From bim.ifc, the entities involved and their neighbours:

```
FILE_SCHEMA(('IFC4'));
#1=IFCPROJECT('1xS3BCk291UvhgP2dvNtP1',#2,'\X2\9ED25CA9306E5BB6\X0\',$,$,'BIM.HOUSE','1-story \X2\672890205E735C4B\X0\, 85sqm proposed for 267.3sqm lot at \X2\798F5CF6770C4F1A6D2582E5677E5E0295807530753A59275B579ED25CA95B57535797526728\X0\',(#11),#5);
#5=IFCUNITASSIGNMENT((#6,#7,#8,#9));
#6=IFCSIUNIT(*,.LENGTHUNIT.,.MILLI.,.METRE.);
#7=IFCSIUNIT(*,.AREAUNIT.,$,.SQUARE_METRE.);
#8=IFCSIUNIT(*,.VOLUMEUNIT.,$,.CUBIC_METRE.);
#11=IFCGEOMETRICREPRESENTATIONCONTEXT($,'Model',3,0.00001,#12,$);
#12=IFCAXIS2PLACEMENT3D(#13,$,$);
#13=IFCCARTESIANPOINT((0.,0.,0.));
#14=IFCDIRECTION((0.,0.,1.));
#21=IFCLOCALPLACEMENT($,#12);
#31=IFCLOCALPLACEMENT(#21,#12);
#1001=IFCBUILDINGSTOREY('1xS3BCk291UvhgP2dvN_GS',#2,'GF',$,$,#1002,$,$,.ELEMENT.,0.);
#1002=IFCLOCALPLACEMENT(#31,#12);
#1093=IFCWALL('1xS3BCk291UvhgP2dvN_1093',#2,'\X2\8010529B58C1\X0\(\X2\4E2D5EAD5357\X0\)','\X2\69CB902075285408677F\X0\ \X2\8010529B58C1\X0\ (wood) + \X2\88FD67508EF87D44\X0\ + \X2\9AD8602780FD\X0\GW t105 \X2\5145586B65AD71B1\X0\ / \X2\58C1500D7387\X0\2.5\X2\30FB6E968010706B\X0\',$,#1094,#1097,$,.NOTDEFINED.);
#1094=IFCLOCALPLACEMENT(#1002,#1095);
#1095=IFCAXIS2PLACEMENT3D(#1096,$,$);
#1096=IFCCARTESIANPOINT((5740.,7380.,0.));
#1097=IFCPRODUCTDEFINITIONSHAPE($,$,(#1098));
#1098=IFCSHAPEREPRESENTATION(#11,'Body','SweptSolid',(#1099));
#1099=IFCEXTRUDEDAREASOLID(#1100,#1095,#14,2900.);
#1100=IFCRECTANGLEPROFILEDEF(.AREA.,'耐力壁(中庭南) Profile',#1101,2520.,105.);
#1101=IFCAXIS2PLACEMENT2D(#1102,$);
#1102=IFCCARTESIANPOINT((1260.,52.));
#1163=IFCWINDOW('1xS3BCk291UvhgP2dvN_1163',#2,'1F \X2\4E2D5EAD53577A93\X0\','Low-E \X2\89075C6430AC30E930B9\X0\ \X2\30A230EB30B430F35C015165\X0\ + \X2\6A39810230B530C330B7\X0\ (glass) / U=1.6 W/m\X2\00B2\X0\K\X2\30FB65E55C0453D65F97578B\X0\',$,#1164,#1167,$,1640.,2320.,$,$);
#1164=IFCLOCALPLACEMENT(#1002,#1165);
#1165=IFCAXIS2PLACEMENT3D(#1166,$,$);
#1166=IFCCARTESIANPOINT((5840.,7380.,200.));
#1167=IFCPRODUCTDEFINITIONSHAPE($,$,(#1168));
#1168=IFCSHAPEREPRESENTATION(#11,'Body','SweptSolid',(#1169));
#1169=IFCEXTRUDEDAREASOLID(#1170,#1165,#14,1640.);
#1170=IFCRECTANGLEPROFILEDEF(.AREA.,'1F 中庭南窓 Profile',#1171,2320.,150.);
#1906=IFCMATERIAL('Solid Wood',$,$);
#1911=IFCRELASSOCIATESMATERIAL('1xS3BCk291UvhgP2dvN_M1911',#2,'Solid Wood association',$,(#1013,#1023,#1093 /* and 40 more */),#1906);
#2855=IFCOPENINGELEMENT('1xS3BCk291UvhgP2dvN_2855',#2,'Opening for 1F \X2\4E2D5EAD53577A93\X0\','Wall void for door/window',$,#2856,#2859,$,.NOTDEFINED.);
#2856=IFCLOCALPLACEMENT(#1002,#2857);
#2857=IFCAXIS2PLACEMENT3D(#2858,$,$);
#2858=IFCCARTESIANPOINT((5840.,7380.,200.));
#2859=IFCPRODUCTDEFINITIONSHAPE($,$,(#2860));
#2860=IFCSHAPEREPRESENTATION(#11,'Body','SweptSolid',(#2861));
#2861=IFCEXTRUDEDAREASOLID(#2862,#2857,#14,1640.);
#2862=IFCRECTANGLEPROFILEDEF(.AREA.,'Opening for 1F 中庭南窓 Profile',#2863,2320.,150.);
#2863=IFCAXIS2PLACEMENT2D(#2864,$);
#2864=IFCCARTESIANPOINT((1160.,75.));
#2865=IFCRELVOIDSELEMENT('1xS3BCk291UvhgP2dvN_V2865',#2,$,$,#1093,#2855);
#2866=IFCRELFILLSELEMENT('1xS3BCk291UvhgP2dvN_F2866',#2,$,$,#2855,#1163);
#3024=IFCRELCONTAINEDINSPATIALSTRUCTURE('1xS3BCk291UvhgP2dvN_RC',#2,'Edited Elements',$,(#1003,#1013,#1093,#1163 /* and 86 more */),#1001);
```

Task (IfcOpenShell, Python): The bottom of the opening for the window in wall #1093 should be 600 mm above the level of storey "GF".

```python
import numpy as np
import ifcopenshell
import ifcopenshell.api.geometry
import ifcopenshell.geom
import ifcopenshell.util.element
import ifcopenshell.util.placement
import ifcopenshell.util.shape
import ifcopenshell.util.unit

model = ifcopenshell.open("bim.ifc")
unit_scale = ifcopenshell.util.unit.calculate_unit_scale(model)

window = model.by_guid("1xS3BCk291UvhgP2dvN_1163")
opening = window.FillsVoids[0].RelatingOpeningElement
storey = ifcopenshell.util.element.get_container(window, ifc_class="IfcBuildingStorey")
level = ifcopenshell.util.placement.get_local_placement(storey.ObjectPlacement)[2, 3]

# The opening's origin need not be at the sill, so measure its lowest point.
shape = ifcopenshell.geom.create_shape(ifcopenshell.geom.settings(), opening)
bottom = ifcopenshell.util.shape.get_shape_bottom_elevation(shape, shape.geometry) / unit_scale
dz = level + 600.0 - bottom

shift = np.array([0.0, 0.0, dz])
# The window is not placed relative to its opening, so move both.
for product in (opening, window):
    matrix = ifcopenshell.util.placement.get_local_placement(product.ObjectPlacement)
    matrix[:3, 3] += shift
    ifcopenshell.api.geometry.edit_object_placement(model, product=product, matrix=matrix, is_si=False)

print(f"moved by {dz * unit_scale:+.3f} m")

model.write("bim_rev.ifc")
```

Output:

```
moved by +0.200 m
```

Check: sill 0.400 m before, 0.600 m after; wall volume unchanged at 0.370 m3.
